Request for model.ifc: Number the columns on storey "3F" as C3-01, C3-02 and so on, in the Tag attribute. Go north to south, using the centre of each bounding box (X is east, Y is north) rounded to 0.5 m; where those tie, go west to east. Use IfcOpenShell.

First a look at what the model holds.

```python
import ifcopenshell
import ifcopenshell.util.element
import ifcopenshell.util.placement

model = ifcopenshell.open("model.ifc")
print(model.schema)
storey = next(s for s in model.by_type("IfcBuildingStorey") if s.Name == "3F")
columns = [e for e in ifcopenshell.util.element.get_decomposition(storey) if e.is_a("IfcColumn")]
for e in sorted(columns, key=lambda e: e.id()):
    origin = ifcopenshell.util.placement.get_local_placement(e.ObjectPlacement)[:3, 3]
    print(e.id(), e.Tag, e.Name, origin.round(2) + 0.0, sep=" | ")
```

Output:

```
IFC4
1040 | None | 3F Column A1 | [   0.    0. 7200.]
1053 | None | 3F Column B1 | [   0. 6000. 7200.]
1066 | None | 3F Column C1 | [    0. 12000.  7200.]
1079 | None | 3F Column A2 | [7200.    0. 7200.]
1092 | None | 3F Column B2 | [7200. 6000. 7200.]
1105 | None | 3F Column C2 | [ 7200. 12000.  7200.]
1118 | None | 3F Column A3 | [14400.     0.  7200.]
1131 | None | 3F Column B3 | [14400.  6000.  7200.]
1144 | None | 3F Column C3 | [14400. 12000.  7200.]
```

```python
import ifcopenshell
import ifcopenshell.geom
import ifcopenshell.util.element
import ifcopenshell.util.shape

model = ifcopenshell.open("model.ifc")
settings = ifcopenshell.geom.settings()
settings.set("use-world-coords", True)


def centre(element):
    shape = ifcopenshell.geom.create_shape(settings, element)
    return ifcopenshell.util.shape.get_bbox_centroid(shape.geometry)


storey = next(s for s in model.by_type("IfcBuildingStorey") if s.Name == "3F")
columns = [e for e in ifcopenshell.util.element.get_decomposition(storey) if e.is_a("IfcColumn")]

# Insertion points can sit at a corner or the storey origin, so sort by the geometry (in metres).
centres = {e: centre(e) for e in columns}
columns.sort(key=lambda e: (-round(centres[e][1] / 0.5), centres[e][0]))

for i, e in enumerate(columns, start=1):
    number = f"C3-{i:02d}"
    e.Tag = number
    print(e.id(), number)

model.write("model_updated.ifc")
```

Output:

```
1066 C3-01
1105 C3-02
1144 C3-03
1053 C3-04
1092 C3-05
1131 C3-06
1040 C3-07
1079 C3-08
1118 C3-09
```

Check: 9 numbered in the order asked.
